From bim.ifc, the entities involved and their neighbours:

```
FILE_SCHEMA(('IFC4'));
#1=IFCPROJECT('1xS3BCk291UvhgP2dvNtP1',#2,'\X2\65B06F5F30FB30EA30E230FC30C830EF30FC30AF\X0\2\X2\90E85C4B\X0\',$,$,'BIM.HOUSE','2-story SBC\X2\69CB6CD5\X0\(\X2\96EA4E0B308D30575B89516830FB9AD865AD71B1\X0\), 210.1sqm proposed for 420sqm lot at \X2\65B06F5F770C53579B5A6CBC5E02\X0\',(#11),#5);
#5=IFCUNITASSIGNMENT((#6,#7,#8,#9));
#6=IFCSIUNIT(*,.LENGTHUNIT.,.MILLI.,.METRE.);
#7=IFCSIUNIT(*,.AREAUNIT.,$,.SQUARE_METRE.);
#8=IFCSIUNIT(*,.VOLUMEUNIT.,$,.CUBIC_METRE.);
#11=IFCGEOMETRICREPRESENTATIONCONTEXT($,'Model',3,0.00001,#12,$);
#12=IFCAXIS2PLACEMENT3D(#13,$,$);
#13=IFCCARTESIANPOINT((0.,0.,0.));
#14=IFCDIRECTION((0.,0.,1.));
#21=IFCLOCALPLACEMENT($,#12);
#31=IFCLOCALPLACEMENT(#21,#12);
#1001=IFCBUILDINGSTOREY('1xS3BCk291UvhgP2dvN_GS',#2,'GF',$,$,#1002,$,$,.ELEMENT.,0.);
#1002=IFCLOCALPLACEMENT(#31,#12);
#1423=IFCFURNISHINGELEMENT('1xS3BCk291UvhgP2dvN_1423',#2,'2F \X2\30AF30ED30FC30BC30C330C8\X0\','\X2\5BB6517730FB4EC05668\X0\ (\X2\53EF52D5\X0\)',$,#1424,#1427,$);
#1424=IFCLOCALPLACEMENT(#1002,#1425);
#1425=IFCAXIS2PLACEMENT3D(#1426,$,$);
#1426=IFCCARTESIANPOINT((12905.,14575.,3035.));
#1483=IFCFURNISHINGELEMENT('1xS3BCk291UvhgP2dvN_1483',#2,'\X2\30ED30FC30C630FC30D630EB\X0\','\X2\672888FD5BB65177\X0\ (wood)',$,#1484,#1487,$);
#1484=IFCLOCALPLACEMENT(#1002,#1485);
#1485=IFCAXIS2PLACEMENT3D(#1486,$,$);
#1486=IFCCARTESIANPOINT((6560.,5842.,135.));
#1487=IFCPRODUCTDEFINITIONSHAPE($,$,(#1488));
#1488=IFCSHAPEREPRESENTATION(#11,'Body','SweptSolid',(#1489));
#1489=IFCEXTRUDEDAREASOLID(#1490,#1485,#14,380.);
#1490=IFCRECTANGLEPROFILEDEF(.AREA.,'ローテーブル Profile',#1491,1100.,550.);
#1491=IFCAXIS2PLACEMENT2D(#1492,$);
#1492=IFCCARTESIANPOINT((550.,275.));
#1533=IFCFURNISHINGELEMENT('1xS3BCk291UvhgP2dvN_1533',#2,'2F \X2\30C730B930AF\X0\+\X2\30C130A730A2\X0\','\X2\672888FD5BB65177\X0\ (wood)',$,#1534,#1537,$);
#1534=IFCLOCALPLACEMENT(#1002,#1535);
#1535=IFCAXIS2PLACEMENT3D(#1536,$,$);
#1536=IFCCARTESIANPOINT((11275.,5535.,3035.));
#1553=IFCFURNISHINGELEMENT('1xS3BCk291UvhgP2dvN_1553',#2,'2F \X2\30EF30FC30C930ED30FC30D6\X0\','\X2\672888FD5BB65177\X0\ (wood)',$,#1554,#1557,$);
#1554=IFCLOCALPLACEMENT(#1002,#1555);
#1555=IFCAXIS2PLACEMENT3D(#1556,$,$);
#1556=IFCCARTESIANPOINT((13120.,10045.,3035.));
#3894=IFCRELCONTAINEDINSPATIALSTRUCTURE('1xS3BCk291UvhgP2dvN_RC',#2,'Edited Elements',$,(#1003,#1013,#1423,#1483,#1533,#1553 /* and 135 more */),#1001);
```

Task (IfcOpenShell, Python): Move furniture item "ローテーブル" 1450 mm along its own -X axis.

```python
import ifcopenshell
import ifcopenshell.api.geometry
import ifcopenshell.util.placement
import ifcopenshell.util.unit

model = ifcopenshell.open("bim.ifc")
unit_scale = ifcopenshell.util.unit.calculate_unit_scale(model)

item = model.by_id(1483)
matrix = ifcopenshell.util.placement.get_local_placement(item.ObjectPlacement)
matrix[:3, 3] -= matrix[:3, 0] * 1.45 / unit_scale
ifcopenshell.api.geometry.edit_object_placement(model, product=item, matrix=matrix, is_si=False)

print(ifcopenshell.util.placement.get_local_placement(item.ObjectPlacement).round(3) + 0.0)

model.write("bim_rev.ifc")
```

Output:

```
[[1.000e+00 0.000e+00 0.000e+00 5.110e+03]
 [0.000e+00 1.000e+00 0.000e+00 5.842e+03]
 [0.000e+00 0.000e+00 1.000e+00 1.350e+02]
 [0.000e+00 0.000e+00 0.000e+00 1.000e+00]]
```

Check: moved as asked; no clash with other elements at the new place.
